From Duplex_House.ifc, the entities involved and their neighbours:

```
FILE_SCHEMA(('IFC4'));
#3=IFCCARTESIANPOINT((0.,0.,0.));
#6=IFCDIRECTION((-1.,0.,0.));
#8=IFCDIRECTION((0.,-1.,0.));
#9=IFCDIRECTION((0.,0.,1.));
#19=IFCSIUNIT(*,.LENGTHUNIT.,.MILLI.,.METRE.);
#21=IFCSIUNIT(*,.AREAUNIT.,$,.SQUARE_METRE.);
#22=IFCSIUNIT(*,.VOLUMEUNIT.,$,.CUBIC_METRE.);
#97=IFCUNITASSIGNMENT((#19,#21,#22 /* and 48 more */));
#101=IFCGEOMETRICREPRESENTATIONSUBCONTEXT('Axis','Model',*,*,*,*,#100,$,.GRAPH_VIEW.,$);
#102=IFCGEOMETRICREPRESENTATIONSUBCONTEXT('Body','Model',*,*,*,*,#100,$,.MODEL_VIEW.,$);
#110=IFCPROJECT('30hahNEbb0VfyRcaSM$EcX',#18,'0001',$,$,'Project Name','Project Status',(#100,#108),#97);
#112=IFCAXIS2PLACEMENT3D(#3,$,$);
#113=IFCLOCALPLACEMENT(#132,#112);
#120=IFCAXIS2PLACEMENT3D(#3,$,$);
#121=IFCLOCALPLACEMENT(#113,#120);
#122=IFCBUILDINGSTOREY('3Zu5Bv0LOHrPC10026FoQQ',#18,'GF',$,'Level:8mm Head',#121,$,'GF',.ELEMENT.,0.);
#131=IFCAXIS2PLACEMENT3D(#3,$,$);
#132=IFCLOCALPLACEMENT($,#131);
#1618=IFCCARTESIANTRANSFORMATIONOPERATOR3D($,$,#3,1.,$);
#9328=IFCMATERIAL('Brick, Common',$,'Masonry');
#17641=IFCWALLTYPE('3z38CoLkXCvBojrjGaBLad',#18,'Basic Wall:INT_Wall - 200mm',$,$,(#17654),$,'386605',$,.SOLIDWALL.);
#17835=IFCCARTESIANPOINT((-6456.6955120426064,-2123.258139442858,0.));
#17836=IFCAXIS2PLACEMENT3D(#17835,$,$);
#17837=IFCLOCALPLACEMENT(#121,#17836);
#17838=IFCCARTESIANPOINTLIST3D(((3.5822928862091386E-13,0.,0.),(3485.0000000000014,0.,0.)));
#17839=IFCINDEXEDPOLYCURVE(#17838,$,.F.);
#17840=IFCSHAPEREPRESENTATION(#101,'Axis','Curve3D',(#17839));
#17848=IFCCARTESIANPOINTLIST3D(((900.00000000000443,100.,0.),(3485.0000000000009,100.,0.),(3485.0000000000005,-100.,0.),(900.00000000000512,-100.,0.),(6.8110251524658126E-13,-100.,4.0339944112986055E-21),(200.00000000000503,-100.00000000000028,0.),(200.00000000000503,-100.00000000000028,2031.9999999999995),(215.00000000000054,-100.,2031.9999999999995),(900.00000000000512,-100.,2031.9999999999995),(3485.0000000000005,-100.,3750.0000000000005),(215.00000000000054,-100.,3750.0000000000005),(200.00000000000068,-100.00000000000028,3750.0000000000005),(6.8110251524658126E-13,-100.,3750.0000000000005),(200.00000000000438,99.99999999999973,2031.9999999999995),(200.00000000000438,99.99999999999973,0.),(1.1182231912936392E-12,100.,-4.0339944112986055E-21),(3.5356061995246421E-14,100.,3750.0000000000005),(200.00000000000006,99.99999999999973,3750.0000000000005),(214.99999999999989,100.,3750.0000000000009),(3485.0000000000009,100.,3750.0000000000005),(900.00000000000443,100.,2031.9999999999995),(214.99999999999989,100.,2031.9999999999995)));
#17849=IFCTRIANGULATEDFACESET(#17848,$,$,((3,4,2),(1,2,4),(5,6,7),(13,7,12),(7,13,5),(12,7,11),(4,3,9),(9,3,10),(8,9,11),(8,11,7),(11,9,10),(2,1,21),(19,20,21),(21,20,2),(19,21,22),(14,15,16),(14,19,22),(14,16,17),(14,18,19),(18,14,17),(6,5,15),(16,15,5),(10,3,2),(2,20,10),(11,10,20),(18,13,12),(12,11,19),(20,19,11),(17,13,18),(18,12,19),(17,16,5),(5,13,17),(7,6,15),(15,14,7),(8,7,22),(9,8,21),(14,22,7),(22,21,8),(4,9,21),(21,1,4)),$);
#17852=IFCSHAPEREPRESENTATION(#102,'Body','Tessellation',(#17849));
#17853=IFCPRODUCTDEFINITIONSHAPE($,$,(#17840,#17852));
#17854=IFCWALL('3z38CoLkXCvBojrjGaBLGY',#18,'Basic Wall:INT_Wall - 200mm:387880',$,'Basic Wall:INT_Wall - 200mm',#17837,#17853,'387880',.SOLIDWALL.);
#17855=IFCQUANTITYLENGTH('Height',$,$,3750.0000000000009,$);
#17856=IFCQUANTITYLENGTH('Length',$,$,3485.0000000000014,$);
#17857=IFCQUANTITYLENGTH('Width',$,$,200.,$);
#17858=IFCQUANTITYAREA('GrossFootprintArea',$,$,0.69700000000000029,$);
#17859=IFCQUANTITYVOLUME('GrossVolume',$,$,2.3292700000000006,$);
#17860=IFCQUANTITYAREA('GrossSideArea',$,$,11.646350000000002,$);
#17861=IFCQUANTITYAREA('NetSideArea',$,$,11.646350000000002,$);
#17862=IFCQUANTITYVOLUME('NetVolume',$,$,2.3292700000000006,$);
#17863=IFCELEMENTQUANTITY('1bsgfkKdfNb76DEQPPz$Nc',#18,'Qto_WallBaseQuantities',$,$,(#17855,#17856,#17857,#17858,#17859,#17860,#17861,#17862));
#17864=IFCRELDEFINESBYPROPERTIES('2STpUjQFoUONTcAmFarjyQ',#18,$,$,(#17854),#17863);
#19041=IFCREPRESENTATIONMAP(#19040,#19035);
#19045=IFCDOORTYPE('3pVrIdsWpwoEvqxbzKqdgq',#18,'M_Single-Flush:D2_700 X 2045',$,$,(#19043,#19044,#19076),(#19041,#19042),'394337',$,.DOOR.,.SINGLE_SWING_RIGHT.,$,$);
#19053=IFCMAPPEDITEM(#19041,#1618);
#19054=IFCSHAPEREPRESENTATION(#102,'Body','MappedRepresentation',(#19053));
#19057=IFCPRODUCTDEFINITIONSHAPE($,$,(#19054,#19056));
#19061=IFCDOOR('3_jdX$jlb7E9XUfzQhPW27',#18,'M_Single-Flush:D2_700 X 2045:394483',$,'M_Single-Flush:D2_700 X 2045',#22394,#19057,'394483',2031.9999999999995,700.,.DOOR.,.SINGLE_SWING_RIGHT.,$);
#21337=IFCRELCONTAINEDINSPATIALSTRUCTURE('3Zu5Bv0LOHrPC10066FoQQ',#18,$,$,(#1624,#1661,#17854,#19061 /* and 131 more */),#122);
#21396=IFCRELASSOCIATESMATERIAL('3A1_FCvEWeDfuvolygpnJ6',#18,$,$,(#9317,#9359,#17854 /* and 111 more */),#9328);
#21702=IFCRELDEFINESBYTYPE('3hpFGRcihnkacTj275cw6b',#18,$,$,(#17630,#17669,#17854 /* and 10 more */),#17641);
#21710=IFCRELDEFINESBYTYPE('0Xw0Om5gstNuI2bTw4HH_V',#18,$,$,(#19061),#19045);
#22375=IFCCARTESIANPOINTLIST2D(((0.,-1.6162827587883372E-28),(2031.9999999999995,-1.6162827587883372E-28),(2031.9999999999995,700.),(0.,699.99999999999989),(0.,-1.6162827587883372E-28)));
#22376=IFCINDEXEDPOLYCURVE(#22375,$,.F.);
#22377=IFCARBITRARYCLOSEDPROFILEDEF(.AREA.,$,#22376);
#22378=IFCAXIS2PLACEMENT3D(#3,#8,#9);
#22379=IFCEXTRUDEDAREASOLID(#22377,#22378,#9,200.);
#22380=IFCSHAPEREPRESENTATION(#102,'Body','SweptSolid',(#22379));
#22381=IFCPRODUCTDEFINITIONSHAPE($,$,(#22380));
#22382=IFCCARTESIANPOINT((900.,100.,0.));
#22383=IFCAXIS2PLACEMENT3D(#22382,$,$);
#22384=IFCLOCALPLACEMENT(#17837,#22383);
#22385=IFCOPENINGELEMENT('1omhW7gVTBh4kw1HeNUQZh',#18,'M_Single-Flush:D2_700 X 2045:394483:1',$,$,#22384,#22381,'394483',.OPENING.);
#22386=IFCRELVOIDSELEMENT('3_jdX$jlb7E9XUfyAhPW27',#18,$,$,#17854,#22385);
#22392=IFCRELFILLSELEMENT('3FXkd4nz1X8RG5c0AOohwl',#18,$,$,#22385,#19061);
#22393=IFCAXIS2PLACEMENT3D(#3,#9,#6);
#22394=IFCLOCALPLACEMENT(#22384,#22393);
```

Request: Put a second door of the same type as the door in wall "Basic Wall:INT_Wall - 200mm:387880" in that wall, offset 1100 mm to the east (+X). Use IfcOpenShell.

```python
import ifcopenshell
import ifcopenshell.api.feature
import ifcopenshell.api.geometry
import ifcopenshell.api.pset
import ifcopenshell.api.root
import ifcopenshell.geom
import ifcopenshell.util.element
import ifcopenshell.util.placement
import ifcopenshell.util.shape
import ifcopenshell.util.unit

model = ifcopenshell.open("Duplex_House.ifc")
area_scale = ifcopenshell.util.unit.calculate_unit_scale(model, "AREAUNIT")
volume_scale = ifcopenshell.util.unit.calculate_unit_scale(model, "VOLUMEUNIT")
settings = ifcopenshell.geom.settings()


def volume(element):
    """Net volume in cubic metres, openings subtracted."""
    shape = ifcopenshell.geom.create_shape(settings, element)
    return ifcopenshell.util.shape.get_volume(shape.geometry)


def reuse_history(source, copy):
    """copy_class also copies each property set's owner history, people and application; keep the originals."""
    for rel in copy.IsDefinedBy:
        if rel.is_a("IfcRelDefinesByProperties") and (history := rel.RelatingPropertyDefinition.OwnerHistory):
            rel.RelatingPropertyDefinition.OwnerHistory = source.OwnerHistory
            ifcopenshell.util.element.remove_deep2(model, history)


door = model.by_id(19061)
opening = door.FillsVoids[0].RelatingOpeningElement
wall = opening.VoidsElements[0].RelatingBuildingElement
before = volume(wall)
shift = ifcopenshell.util.placement.get_local_placement(wall.ObjectPlacement)[:3, 0] * 1100.0

# copy_class copies the void relationship, type, container and properties, but no geometry.
new_opening = ifcopenshell.api.root.copy_class(model, product=opening)
new_opening.Representation = ifcopenshell.util.element.copy_deep(
    model, opening.Representation, exclude=["IfcGeometricRepresentationContext", "IfcRepresentationMap"]
)
new_opening.Name = "M_Single-Flush:D2_700 X 2045"
new_opening.Tag = None
reuse_history(opening, new_opening)
new_door = ifcopenshell.api.root.copy_class(model, product=door)
new_door.Representation = ifcopenshell.util.element.copy_deep(
    model, door.Representation, exclude=["IfcGeometricRepresentationContext", "IfcRepresentationMap"]
)
new_door.Name = "M_Single-Flush:D2_700 X 2045"
new_door.Tag = None
reuse_history(door, new_door)
ifcopenshell.api.feature.add_filling(model, opening=new_opening, element=new_door)

for old, new in ((opening, new_opening), (door, new_door)):
    matrix = ifcopenshell.util.placement.get_local_placement(old.ObjectPlacement)
    matrix[:3, 3] += shift
    ifcopenshell.api.geometry.edit_object_placement(model, product=new, matrix=matrix, is_si=False)

after = volume(wall)
thickness = 0.2  # wall thickness in metres

# Update the wall's stored quantities.
qto = model.by_id(ifcopenshell.util.element.get_pset(wall, "Qto_WallBaseQuantities", should_inherit=False)["id"])
ifcopenshell.api.pset.edit_qto(model, qto=qto, properties={
    "NetSideArea": after / thickness / area_scale,
    "NetVolume": after / volume_scale,
})

print(f"wall volume {before:.3f} -> {after:.3f} m3")

model.write("Duplex_House_v2.ifc")
```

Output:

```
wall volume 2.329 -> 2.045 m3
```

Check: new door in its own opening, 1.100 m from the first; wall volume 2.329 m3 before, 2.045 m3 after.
